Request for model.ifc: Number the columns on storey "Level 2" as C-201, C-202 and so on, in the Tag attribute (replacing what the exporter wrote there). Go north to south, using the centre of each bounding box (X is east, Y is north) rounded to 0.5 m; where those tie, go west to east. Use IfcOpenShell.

First a look at what the model holds.

```python
import ifcopenshell
import ifcopenshell.util.element
import ifcopenshell.util.placement

model = ifcopenshell.open("model.ifc")
print(model.schema)
storey = next(s for s in model.by_type("IfcBuildingStorey") if s.Name == "Level 2")
columns = [e for e in ifcopenshell.util.element.get_decomposition(storey) if e.is_a("IfcColumn")]
for e in sorted(columns, key=lambda e: e.id()):
    origin = ifcopenshell.util.placement.get_local_placement(e.ObjectPlacement)[:3, 3]
    print(e.id(), e.Tag, e.Name, origin.round(2) + 0.0, sep=" | ")
```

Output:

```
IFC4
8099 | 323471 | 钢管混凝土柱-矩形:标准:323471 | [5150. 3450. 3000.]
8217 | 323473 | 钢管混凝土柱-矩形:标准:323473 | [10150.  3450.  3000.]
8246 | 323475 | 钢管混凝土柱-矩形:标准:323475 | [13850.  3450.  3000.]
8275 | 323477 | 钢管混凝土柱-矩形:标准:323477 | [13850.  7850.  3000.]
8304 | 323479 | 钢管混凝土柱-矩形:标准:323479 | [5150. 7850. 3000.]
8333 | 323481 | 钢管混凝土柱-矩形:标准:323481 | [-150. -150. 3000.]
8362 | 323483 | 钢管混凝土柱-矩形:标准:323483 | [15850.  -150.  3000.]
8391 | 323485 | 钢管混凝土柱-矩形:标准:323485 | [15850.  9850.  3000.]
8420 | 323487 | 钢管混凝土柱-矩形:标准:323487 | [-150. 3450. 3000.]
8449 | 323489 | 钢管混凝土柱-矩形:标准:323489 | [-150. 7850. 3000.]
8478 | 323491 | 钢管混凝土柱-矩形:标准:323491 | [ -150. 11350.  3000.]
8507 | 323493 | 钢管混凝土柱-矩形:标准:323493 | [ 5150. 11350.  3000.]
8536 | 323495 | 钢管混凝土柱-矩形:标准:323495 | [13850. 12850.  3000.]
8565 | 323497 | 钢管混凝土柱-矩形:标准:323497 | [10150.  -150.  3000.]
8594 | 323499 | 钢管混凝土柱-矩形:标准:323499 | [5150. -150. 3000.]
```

```python
import ifcopenshell
import ifcopenshell.geom
import ifcopenshell.util.element
import ifcopenshell.util.shape

model = ifcopenshell.open("model.ifc")
settings = ifcopenshell.geom.settings()
settings.set("use-world-coords", True)


def centre(element):
    shape = ifcopenshell.geom.create_shape(settings, element)
    return ifcopenshell.util.shape.get_bbox_centroid(shape.geometry)


storey = next(s for s in model.by_type("IfcBuildingStorey") if s.Name == "Level 2")
columns = [e for e in ifcopenshell.util.element.get_decomposition(storey) if e.is_a("IfcColumn")]

# Insertion points can sit at a corner or the storey origin, so sort by the geometry (in metres).
centres = {e: centre(e) for e in columns}
columns.sort(key=lambda e: (-round(centres[e][1] / 0.5), centres[e][0]))

for i, e in enumerate(columns, start=1):
    number = f"C-2{i:02d}"
    e.Tag = number
    print(e.id(), number)

model.write("model_rev.ifc")
```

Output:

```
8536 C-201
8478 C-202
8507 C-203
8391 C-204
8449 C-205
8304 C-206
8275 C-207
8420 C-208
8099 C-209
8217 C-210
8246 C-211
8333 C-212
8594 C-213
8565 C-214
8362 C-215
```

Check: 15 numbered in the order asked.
